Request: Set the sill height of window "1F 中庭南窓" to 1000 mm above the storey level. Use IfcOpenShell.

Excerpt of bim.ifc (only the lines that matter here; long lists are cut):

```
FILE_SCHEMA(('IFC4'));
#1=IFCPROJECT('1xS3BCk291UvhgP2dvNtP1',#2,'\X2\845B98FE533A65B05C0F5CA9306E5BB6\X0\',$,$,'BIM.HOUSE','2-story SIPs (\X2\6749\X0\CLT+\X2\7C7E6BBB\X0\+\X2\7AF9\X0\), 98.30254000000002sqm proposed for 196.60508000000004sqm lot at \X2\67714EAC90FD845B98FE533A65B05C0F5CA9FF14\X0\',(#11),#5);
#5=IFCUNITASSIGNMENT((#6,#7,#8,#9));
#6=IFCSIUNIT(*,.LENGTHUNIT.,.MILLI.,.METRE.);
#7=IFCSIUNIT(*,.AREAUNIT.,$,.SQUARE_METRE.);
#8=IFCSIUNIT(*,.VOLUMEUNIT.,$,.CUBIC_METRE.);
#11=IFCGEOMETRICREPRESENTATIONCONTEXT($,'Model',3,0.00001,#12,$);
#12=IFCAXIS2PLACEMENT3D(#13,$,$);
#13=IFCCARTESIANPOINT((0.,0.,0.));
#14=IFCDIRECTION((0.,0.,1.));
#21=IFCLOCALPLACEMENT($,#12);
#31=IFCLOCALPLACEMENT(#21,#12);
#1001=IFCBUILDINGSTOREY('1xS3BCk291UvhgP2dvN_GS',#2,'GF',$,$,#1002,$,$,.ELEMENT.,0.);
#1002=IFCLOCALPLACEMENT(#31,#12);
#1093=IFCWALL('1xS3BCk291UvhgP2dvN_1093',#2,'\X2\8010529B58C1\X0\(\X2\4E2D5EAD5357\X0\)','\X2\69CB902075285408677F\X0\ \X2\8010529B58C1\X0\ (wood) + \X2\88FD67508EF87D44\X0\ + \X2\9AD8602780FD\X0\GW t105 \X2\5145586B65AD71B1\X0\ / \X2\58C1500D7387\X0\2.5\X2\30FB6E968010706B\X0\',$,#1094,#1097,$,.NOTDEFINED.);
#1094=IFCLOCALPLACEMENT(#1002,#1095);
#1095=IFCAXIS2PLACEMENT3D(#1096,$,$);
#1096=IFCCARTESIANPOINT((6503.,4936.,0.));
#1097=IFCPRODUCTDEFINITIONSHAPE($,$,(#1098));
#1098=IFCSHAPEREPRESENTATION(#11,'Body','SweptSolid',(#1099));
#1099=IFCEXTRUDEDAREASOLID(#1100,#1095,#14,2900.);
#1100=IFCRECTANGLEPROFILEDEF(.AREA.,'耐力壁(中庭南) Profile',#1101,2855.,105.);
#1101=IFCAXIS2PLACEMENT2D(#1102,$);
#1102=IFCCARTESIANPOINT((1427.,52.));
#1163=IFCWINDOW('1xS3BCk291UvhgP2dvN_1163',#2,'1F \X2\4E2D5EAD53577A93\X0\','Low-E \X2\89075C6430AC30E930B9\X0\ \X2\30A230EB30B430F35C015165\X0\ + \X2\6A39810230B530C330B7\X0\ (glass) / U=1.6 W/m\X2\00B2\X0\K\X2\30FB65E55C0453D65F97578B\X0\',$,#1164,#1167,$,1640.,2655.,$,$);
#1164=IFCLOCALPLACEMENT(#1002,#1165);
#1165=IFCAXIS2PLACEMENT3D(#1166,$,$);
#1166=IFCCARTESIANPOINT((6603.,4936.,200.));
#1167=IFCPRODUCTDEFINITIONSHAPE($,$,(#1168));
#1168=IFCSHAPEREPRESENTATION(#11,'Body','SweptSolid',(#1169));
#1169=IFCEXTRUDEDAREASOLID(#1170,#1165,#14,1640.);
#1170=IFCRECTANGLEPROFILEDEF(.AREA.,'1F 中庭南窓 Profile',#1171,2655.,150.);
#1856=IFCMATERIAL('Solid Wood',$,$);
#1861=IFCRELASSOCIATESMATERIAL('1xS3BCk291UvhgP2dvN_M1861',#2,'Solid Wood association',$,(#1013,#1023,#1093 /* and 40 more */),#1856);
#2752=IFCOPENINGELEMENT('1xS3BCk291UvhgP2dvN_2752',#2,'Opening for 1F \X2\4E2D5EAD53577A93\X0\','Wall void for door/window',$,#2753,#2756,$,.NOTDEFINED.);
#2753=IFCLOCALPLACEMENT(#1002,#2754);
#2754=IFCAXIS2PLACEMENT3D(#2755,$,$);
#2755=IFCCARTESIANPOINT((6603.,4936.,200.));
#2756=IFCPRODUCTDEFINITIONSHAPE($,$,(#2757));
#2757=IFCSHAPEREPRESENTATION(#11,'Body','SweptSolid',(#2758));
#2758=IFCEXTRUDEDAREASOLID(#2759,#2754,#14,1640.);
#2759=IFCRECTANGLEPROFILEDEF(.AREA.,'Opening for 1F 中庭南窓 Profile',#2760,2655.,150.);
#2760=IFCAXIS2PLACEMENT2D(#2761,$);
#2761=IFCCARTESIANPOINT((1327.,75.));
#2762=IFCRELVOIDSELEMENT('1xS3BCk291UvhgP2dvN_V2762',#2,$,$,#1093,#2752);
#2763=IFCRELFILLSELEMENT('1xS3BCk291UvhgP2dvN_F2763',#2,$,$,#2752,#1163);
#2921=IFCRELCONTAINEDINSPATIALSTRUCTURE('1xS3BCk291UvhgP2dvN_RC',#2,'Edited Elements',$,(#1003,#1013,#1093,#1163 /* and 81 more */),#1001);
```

```python
import numpy as np
import ifcopenshell
import ifcopenshell.api.geometry
import ifcopenshell.geom
import ifcopenshell.util.element
import ifcopenshell.util.placement
import ifcopenshell.util.shape
import ifcopenshell.util.unit

model = ifcopenshell.open("bim.ifc")
unit_scale = ifcopenshell.util.unit.calculate_unit_scale(model)

window = model.by_guid("1xS3BCk291UvhgP2dvN_1163")
opening = window.FillsVoids[0].RelatingOpeningElement
storey = ifcopenshell.util.element.get_container(window, ifc_class="IfcBuildingStorey")
level = ifcopenshell.util.placement.get_local_placement(storey.ObjectPlacement)[2, 3]

# The opening's origin need not be at the sill, so measure its lowest point.
shape = ifcopenshell.geom.create_shape(ifcopenshell.geom.settings(), opening)
bottom = ifcopenshell.util.shape.get_shape_bottom_elevation(shape, shape.geometry) / unit_scale
dz = level + 1000.0 - bottom

shift = np.array([0.0, 0.0, dz])
# The window is not placed relative to its opening, so move both.
for product in (opening, window):
    matrix = ifcopenshell.util.placement.get_local_placement(product.ObjectPlacement)
    matrix[:3, 3] += shift
    ifcopenshell.api.geometry.edit_object_placement(model, product=product, matrix=matrix, is_si=False)

print(f"moved by {dz * unit_scale:+.3f} m")

model.write("bim_rev.ifc")
```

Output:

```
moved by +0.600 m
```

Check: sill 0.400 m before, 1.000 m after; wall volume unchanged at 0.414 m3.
